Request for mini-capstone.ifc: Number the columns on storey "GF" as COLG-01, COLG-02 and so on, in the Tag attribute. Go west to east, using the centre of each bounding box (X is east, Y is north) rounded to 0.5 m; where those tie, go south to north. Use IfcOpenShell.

First a look at what the model holds.

```python
import ifcopenshell
import ifcopenshell.util.element
import ifcopenshell.util.placement

model = ifcopenshell.open("mini-capstone.ifc")
print(model.schema)
storey = next(s for s in model.by_type("IfcBuildingStorey") if s.Name == "GF")
columns = [e for e in ifcopenshell.util.element.get_decomposition(storey) if e.is_a("IfcColumn")]
for e in sorted(columns, key=lambda e: e.id()):
    origin = ifcopenshell.util.placement.get_local_placement(e.ObjectPlacement)[:3, 3]
    print(e.id(), e.Tag, e.Name, origin.round(2) + 0.0, sep=" | ")
```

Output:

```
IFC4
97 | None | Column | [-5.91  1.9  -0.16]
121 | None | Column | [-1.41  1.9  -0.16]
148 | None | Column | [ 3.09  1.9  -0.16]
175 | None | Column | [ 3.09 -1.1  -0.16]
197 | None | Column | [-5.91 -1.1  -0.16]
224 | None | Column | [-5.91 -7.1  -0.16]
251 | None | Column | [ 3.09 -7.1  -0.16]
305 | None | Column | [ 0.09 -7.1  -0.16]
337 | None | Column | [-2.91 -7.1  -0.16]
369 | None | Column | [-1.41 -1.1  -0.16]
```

```python
import ifcopenshell
import ifcopenshell.geom
import ifcopenshell.util.element
import ifcopenshell.util.shape

model = ifcopenshell.open("mini-capstone.ifc")
settings = ifcopenshell.geom.settings()
settings.set("use-world-coords", True)


def centre(element):
    shape = ifcopenshell.geom.create_shape(settings, element)
    return ifcopenshell.util.shape.get_bbox_centroid(shape.geometry)


storey = next(s for s in model.by_type("IfcBuildingStorey") if s.Name == "GF")
columns = [e for e in ifcopenshell.util.element.get_decomposition(storey) if e.is_a("IfcColumn")]

# Insertion points can sit at a corner or the storey origin, so sort by the geometry (in metres).
centres = {e: centre(e) for e in columns}
columns.sort(key=lambda e: (round(centres[e][0] / 0.5), centres[e][1]))

for i, e in enumerate(columns, start=1):
    number = f"COLG-{i:02d}"
    e.Tag = number
    print(e.id(), number)

model.write("mini-capstone_rev.ifc")
```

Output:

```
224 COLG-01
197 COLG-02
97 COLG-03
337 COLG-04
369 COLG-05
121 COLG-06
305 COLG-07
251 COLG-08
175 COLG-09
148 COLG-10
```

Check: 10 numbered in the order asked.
